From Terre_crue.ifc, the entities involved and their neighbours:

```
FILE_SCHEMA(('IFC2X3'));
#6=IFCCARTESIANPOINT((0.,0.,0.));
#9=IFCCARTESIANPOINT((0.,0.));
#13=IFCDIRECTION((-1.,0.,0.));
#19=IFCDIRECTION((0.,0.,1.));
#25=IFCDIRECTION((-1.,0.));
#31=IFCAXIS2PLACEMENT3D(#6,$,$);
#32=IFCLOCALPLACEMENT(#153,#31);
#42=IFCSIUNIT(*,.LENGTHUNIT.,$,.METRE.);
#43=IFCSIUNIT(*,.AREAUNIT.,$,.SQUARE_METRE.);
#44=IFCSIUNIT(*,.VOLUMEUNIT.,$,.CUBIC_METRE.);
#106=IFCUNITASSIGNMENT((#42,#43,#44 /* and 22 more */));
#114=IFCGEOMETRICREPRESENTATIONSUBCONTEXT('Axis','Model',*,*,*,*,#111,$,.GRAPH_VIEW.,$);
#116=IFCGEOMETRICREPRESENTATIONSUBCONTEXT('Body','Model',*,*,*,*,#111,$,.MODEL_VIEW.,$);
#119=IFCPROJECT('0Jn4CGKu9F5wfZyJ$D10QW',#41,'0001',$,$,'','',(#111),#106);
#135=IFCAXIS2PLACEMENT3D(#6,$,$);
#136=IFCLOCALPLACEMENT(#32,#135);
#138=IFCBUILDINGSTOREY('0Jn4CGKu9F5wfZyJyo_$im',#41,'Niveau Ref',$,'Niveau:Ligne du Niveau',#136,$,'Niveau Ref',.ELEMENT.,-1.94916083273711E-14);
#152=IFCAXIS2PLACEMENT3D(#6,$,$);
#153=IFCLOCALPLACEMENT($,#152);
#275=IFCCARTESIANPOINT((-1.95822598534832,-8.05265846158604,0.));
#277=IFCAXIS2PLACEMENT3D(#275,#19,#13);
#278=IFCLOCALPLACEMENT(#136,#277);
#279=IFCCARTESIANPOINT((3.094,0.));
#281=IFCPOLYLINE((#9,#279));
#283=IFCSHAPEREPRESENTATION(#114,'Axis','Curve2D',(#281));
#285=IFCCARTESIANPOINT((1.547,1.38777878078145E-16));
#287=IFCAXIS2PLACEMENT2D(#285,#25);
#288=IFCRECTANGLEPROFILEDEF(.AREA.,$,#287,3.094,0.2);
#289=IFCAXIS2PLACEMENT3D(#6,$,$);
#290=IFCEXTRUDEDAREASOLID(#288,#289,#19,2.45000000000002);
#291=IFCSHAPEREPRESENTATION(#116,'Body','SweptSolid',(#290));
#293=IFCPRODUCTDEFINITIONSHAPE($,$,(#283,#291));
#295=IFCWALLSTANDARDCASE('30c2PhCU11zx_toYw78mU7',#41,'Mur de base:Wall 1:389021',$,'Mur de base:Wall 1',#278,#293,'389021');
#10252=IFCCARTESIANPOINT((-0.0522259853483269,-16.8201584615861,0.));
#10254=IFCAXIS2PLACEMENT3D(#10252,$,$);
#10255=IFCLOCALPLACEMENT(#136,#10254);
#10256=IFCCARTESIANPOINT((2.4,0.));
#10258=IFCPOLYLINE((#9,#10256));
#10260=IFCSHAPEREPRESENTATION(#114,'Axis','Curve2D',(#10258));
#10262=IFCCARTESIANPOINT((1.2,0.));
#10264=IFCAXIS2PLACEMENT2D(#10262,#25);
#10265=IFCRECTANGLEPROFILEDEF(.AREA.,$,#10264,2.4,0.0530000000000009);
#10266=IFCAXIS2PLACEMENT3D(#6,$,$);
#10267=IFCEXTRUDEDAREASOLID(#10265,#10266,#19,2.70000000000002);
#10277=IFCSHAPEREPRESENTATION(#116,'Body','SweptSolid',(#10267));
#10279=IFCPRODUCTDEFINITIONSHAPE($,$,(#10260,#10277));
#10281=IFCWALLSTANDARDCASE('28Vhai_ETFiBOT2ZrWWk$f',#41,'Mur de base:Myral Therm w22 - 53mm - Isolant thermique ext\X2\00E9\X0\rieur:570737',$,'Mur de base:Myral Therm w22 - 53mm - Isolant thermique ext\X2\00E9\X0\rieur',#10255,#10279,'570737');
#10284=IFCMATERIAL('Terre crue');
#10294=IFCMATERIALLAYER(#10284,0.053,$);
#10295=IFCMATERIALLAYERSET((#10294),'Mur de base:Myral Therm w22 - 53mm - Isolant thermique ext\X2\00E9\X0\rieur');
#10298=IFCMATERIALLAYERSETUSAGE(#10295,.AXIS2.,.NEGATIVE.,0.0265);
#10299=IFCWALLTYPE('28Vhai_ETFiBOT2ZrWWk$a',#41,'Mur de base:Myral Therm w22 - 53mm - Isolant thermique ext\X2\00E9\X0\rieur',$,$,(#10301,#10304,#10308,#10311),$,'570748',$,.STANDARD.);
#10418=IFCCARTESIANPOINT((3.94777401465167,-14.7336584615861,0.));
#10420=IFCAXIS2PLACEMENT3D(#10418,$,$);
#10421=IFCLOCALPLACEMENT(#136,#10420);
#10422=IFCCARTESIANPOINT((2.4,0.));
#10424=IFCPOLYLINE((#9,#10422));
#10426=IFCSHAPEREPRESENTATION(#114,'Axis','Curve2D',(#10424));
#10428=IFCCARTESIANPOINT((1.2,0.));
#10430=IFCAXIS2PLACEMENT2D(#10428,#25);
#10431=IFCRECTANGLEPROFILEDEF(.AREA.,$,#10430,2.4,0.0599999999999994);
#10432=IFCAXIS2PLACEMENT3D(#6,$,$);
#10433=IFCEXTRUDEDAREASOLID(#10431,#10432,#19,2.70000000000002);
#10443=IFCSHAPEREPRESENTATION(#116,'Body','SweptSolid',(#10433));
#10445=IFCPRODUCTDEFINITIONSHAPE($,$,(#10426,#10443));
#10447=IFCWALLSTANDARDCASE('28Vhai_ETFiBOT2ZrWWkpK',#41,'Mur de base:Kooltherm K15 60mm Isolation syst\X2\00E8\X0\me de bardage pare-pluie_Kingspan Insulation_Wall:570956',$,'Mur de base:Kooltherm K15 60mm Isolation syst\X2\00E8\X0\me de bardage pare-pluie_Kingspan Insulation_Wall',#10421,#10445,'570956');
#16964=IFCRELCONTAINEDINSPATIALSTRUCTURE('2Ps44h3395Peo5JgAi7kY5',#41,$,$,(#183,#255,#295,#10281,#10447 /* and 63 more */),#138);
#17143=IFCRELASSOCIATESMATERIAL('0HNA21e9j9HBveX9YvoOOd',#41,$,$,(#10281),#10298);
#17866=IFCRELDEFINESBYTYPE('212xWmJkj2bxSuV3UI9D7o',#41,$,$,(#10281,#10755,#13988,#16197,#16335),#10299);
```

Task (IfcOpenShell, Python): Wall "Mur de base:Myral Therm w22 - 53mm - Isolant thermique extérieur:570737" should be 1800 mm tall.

```python
import ifcopenshell
import ifcopenshell.geom
import ifcopenshell.util.representation
import ifcopenshell.util.shape

model = ifcopenshell.open("Terre_crue.ifc")
settings = ifcopenshell.geom.settings()


def volume(element):
    """Net volume in cubic metres, openings subtracted."""
    shape = ifcopenshell.geom.create_shape(settings, element)
    return ifcopenshell.util.shape.get_volume(shape.geometry)


wall = model.by_guid("28Vhai_ETFiBOT2ZrWWk$f")
before = volume(wall)

body = ifcopenshell.util.representation.get_representation(wall, "Model", "Body")
solid = body.Items[0]
old_height = solid.Depth
solid.Depth = 1.8
after = volume(wall)

print(f"height {old_height:g} -> {solid.Depth:g}, volume {before:.3f} -> {after:.3f} m3")

model.write("Terre_crue_edited.ifc")
```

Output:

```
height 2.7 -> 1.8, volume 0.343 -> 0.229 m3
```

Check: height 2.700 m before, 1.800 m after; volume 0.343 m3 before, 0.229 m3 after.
